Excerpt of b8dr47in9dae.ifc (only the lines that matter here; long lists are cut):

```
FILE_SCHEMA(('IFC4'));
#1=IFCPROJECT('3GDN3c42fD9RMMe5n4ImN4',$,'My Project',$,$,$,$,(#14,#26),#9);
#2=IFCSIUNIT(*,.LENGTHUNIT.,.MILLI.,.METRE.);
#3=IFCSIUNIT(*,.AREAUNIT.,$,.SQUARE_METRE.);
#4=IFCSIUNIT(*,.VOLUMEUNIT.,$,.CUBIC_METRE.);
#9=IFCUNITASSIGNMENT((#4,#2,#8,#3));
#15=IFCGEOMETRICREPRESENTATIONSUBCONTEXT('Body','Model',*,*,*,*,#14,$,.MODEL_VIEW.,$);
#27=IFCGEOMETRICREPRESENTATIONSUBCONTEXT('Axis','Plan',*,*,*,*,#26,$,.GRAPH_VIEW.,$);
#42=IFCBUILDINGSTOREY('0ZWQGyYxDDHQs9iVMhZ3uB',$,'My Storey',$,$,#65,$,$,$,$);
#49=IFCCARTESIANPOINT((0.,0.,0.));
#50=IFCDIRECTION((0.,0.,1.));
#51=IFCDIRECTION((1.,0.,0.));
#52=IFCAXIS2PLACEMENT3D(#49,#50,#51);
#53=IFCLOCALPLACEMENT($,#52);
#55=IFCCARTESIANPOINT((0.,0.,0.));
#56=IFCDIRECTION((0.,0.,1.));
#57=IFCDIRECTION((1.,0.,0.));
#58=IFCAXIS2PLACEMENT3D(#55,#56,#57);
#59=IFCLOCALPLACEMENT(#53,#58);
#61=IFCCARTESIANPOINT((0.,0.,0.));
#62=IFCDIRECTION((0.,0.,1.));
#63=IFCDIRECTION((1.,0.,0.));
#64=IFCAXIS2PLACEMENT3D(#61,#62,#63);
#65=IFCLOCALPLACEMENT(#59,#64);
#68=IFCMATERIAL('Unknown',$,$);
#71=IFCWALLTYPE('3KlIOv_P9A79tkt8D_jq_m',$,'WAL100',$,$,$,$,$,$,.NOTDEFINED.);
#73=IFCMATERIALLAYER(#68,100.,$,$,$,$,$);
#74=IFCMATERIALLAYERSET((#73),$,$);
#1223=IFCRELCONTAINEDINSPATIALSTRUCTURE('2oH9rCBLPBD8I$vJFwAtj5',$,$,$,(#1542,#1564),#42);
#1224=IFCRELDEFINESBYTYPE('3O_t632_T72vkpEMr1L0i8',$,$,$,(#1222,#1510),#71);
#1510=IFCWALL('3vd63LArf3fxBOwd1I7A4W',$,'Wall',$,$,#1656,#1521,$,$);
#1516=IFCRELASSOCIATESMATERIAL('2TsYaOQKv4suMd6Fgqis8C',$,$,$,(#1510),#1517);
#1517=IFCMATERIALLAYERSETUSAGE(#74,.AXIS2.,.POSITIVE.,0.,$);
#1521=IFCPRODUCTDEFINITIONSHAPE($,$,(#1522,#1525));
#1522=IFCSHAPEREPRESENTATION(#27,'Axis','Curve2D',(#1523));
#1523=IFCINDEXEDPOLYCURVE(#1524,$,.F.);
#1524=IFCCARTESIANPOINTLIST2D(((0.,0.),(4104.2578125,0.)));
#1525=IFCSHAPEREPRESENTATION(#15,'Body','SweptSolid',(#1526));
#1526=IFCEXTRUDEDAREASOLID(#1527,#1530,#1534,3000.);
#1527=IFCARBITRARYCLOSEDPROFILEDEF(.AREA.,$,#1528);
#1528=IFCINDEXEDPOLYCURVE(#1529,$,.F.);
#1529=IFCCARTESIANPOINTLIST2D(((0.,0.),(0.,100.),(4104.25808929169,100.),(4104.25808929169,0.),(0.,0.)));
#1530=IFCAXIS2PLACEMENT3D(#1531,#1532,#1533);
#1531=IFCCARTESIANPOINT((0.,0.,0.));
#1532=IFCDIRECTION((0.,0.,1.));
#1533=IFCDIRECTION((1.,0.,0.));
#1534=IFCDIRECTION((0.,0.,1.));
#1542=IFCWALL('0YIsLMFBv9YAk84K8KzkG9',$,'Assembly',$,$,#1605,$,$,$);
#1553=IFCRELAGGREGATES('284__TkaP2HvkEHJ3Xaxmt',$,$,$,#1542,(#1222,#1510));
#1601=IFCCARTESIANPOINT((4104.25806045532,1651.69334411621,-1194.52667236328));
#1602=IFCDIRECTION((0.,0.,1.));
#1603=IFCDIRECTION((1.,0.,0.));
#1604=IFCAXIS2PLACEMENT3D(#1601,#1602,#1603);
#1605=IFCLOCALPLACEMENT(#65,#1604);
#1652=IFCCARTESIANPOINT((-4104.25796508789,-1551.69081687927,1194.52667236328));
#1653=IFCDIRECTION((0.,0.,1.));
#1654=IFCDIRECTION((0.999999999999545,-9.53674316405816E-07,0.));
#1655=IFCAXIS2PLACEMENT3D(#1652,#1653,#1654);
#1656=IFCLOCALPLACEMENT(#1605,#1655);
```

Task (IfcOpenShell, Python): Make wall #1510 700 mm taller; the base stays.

```python
import ifcopenshell
import ifcopenshell.geom
import ifcopenshell.util.representation
import ifcopenshell.util.shape
import ifcopenshell.util.unit

model = ifcopenshell.open("b8dr47in9dae.ifc")
unit_scale = ifcopenshell.util.unit.calculate_unit_scale(model)
settings = ifcopenshell.geom.settings()


def volume(element):
    """Net volume in cubic metres, openings subtracted."""
    shape = ifcopenshell.geom.create_shape(settings, element)
    return ifcopenshell.util.shape.get_volume(shape.geometry)


wall = model.by_guid("3vd63LArf3fxBOwd1I7A4W")
before = volume(wall)

body = ifcopenshell.util.representation.get_representation(wall, "Model", "Body")
solid = body.Items[0]
old_height = solid.Depth
solid.Depth += 0.7 / unit_scale
after = volume(wall)

print(f"height {old_height:g} -> {solid.Depth:g}, volume {before:.3f} -> {after:.3f} m3")

model.write("b8dr47in9dae_v2.ifc")
```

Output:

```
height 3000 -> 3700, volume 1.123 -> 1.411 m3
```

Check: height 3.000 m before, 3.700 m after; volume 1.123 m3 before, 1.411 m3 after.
